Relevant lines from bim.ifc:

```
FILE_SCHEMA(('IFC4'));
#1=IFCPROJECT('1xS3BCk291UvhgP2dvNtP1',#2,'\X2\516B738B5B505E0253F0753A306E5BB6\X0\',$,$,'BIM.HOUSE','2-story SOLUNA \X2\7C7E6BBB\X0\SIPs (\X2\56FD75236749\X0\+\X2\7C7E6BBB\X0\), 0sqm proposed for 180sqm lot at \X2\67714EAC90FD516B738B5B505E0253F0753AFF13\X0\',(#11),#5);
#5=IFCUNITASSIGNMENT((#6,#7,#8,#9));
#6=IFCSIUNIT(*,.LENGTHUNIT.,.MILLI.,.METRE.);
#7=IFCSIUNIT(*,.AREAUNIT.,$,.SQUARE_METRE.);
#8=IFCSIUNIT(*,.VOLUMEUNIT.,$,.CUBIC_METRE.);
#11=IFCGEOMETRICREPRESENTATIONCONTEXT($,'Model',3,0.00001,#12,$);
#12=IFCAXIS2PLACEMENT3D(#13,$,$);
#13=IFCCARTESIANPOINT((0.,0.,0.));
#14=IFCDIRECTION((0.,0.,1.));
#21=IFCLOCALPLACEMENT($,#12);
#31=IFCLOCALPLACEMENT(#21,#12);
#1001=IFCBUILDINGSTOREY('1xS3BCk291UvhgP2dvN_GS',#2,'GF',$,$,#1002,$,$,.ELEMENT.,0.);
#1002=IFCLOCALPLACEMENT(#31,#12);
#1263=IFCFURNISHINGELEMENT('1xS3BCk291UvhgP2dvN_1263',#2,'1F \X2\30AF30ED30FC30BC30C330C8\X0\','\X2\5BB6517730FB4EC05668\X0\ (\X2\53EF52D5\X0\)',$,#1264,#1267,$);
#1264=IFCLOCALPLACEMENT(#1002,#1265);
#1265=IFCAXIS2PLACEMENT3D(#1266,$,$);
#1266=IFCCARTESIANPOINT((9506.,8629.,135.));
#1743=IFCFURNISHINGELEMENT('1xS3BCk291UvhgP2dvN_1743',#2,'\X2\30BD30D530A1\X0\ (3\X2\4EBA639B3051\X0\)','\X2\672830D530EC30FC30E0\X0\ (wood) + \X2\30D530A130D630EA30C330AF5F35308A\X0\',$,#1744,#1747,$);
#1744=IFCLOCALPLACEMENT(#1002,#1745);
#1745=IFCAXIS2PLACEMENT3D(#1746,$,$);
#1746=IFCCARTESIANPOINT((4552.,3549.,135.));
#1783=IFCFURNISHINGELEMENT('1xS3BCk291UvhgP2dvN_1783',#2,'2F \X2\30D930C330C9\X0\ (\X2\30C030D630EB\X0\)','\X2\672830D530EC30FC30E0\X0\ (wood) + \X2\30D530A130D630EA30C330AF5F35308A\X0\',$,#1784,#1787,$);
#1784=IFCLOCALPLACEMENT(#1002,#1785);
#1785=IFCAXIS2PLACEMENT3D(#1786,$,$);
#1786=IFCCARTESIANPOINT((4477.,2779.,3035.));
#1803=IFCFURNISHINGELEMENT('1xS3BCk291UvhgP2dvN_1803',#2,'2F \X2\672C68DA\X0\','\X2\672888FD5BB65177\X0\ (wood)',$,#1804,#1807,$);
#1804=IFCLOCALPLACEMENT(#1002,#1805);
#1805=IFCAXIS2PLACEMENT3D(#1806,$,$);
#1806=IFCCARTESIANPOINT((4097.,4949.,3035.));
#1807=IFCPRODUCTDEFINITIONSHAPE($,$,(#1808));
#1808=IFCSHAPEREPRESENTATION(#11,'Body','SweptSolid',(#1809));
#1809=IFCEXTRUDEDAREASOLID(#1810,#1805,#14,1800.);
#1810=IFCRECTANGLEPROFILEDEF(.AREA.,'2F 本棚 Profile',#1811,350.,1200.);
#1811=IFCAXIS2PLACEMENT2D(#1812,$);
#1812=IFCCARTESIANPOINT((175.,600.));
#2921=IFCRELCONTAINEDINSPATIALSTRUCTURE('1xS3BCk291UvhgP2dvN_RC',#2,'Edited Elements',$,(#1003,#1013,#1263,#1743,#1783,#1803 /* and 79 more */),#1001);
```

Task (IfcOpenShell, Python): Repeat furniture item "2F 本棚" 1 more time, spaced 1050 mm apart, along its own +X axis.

```python
import ifcopenshell
import ifcopenshell.api.geometry
import ifcopenshell.api.root
import ifcopenshell.util.element
import ifcopenshell.util.placement

model = ifcopenshell.open("bim.ifc")


def reuse_history(source, copy):
    """copy_class also copies each property set's owner history, people and application; keep the originals."""
    for rel in copy.IsDefinedBy:
        if rel.is_a("IfcRelDefinesByProperties") and (history := rel.RelatingPropertyDefinition.OwnerHistory):
            rel.RelatingPropertyDefinition.OwnerHistory = source.OwnerHistory
            ifcopenshell.util.element.remove_deep2(model, history)


source = model.by_guid("1xS3BCk291UvhgP2dvN_1803")
base = ifcopenshell.util.placement.get_local_placement(source.ObjectPlacement)
step = base[:3, 0] * 1050.0

for i in range(1, 2):
    copy = ifcopenshell.api.root.copy_class(model, product=source)
    copy.Representation = ifcopenshell.util.element.copy_deep(
        model, source.Representation, exclude=["IfcGeometricRepresentationContext", "IfcRepresentationMap"]
    )
    reuse_history(source, copy)
    matrix = base.copy()
    matrix[:3, 3] += i * step
    print("added at", matrix[:3, 3].round(3) + 0.0)
    ifcopenshell.api.geometry.edit_object_placement(model, product=copy, matrix=matrix, is_si=False)

model.write("bim_v2.ifc")
```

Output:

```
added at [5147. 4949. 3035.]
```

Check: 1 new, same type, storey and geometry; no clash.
